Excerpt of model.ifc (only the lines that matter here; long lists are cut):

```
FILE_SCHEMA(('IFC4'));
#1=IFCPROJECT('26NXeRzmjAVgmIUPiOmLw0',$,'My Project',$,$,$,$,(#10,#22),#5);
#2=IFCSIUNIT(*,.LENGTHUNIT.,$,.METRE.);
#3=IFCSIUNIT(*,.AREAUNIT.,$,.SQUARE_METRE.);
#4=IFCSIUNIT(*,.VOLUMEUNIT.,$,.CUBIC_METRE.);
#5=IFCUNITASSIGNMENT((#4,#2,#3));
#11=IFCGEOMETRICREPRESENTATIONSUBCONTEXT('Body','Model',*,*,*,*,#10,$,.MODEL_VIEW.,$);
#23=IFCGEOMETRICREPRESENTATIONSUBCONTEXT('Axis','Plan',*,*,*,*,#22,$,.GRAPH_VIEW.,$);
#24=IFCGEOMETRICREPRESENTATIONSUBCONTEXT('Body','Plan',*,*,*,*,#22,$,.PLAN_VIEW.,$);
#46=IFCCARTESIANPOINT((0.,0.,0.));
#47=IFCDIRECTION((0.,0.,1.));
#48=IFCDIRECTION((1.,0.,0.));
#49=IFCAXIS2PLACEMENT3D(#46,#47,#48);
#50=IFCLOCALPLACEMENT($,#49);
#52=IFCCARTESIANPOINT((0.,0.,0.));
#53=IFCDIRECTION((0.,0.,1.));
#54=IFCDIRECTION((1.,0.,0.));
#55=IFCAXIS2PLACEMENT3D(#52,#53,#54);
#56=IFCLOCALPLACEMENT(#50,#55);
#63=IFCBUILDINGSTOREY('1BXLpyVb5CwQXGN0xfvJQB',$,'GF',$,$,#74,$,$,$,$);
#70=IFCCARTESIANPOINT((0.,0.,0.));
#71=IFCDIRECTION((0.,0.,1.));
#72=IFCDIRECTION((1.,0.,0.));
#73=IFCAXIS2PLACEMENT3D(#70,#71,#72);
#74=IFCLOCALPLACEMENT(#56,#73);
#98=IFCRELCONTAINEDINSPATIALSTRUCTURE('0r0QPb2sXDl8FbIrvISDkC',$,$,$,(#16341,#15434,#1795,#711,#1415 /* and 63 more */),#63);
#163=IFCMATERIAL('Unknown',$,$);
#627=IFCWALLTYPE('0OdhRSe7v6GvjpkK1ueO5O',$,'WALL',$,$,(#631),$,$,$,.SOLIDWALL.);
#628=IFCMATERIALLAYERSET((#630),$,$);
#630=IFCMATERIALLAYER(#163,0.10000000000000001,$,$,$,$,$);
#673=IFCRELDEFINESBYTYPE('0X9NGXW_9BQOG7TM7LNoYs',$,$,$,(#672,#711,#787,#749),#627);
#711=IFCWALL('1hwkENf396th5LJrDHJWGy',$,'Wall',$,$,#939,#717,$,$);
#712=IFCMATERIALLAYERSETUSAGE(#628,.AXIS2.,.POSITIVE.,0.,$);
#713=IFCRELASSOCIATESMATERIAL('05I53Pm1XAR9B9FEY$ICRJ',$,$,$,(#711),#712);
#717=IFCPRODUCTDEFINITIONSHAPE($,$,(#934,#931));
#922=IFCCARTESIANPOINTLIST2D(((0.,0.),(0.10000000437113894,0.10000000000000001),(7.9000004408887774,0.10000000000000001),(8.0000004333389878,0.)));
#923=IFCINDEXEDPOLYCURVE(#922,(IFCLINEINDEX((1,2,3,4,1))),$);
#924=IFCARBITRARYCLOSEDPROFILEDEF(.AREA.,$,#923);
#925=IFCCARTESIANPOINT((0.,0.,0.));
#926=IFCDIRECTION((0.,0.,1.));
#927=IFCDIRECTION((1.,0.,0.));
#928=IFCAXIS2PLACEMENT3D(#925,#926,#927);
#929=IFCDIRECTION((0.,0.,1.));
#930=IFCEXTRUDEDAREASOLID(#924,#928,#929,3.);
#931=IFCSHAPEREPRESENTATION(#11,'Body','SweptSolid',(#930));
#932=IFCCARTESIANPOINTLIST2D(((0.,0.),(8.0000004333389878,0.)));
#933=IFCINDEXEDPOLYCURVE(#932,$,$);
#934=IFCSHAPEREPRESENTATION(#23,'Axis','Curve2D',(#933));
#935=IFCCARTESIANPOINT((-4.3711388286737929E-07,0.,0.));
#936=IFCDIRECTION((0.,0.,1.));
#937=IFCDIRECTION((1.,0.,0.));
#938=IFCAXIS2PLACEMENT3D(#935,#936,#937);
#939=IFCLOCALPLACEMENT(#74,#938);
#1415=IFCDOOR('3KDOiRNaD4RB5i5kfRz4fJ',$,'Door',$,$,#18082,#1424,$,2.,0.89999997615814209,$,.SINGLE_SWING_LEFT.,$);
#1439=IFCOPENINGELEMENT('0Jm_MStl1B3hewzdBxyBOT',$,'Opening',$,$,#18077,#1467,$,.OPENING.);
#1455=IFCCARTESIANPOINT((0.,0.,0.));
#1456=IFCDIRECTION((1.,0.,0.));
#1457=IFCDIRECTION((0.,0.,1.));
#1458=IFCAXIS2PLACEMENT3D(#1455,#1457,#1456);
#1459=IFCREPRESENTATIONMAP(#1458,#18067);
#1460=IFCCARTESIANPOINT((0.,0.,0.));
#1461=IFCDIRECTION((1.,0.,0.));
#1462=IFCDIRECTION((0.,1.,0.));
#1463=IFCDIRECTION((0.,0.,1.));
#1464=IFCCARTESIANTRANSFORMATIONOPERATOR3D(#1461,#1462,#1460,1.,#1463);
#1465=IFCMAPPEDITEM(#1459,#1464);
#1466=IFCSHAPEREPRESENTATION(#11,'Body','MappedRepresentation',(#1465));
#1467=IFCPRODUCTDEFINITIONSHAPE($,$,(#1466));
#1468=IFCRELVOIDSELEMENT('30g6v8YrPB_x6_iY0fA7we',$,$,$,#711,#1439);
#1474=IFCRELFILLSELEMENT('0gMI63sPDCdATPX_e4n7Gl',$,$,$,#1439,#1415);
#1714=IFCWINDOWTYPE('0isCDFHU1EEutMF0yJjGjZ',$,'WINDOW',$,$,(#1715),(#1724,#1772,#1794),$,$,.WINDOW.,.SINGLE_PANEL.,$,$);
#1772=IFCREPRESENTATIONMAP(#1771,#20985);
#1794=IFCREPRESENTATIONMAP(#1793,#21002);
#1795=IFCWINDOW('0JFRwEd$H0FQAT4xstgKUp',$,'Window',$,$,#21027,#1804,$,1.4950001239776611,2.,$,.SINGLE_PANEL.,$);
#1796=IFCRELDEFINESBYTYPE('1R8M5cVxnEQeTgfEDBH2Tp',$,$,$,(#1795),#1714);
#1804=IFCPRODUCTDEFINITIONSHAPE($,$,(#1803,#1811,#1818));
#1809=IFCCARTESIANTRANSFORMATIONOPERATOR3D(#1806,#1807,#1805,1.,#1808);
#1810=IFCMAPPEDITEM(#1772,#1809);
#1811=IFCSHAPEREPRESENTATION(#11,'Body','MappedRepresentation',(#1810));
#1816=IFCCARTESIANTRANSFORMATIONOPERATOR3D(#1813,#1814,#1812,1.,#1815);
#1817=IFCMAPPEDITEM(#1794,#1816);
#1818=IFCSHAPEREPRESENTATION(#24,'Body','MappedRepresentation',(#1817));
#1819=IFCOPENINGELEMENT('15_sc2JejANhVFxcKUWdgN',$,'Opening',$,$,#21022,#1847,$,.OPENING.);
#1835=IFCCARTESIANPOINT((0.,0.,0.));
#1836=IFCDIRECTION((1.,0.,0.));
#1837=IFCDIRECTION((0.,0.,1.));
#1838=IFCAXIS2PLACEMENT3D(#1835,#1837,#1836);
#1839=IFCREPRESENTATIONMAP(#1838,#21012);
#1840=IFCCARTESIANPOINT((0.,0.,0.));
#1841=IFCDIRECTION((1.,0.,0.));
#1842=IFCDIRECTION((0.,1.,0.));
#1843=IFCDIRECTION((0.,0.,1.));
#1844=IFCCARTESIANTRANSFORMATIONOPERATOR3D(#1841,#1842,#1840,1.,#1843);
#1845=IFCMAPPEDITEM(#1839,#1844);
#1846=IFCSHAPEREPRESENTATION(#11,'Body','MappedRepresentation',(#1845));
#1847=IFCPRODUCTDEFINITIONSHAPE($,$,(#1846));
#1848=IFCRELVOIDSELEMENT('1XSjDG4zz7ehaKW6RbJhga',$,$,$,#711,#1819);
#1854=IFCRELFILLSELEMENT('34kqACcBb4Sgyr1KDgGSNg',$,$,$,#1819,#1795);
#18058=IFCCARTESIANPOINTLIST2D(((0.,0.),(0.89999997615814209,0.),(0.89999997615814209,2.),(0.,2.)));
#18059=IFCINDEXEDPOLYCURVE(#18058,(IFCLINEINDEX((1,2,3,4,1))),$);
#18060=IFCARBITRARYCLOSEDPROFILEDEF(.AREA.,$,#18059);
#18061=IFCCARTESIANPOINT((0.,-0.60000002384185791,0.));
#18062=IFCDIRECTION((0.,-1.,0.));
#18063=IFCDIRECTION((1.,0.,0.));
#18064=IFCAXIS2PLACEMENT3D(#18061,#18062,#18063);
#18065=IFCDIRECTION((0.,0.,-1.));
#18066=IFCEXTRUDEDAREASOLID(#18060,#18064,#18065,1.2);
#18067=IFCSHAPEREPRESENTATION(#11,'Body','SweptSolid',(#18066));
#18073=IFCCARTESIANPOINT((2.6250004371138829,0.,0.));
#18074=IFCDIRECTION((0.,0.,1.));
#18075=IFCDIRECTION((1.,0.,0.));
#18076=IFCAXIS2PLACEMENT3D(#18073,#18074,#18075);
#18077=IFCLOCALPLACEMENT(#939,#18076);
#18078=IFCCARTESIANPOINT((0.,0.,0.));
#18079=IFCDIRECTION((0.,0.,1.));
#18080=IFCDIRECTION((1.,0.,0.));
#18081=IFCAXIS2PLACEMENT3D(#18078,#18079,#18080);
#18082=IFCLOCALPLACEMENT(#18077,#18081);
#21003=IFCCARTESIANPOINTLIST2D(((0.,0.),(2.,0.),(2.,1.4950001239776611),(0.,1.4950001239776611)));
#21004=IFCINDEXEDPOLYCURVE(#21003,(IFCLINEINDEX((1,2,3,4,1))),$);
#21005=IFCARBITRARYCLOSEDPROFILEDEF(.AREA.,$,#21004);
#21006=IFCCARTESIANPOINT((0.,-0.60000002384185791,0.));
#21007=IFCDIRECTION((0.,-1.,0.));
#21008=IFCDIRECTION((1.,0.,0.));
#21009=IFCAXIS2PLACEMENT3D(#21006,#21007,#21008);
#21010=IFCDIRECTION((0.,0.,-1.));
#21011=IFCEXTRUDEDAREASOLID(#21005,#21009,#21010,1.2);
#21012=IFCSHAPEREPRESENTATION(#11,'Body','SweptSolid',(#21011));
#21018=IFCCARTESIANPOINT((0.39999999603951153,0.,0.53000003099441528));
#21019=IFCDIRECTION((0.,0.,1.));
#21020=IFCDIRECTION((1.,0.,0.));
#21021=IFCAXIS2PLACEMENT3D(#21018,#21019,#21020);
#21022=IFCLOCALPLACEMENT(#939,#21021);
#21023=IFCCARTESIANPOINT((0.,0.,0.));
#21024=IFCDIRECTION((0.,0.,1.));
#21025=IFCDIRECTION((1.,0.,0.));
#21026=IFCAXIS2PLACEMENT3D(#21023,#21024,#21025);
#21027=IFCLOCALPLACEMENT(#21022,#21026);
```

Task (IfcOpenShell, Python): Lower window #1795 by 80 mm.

```python
import numpy as np
import ifcopenshell
import ifcopenshell.api.geometry
import ifcopenshell.util.placement
import ifcopenshell.util.unit

model = ifcopenshell.open("model.ifc")
unit_scale = ifcopenshell.util.unit.calculate_unit_scale(model)

window = model.by_guid("0JFRwEd$H0FQAT4xstgKUp")
opening = window.FillsVoids[0].RelatingOpeningElement
dz = -0.08 / unit_scale

shift = np.array([0.0, 0.0, dz])
# The window is placed relative to its opening, so it follows when the opening moves.
matrix = ifcopenshell.util.placement.get_local_placement(opening.ObjectPlacement)
matrix[:3, 3] += shift
ifcopenshell.api.geometry.edit_object_placement(
    model, product=opening, matrix=matrix, is_si=False, should_transform_children=True
)

print(f"moved by {dz * unit_scale:+.3f} m")

model.write("model_rev.ifc")
```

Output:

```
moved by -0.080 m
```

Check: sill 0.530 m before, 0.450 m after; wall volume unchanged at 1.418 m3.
